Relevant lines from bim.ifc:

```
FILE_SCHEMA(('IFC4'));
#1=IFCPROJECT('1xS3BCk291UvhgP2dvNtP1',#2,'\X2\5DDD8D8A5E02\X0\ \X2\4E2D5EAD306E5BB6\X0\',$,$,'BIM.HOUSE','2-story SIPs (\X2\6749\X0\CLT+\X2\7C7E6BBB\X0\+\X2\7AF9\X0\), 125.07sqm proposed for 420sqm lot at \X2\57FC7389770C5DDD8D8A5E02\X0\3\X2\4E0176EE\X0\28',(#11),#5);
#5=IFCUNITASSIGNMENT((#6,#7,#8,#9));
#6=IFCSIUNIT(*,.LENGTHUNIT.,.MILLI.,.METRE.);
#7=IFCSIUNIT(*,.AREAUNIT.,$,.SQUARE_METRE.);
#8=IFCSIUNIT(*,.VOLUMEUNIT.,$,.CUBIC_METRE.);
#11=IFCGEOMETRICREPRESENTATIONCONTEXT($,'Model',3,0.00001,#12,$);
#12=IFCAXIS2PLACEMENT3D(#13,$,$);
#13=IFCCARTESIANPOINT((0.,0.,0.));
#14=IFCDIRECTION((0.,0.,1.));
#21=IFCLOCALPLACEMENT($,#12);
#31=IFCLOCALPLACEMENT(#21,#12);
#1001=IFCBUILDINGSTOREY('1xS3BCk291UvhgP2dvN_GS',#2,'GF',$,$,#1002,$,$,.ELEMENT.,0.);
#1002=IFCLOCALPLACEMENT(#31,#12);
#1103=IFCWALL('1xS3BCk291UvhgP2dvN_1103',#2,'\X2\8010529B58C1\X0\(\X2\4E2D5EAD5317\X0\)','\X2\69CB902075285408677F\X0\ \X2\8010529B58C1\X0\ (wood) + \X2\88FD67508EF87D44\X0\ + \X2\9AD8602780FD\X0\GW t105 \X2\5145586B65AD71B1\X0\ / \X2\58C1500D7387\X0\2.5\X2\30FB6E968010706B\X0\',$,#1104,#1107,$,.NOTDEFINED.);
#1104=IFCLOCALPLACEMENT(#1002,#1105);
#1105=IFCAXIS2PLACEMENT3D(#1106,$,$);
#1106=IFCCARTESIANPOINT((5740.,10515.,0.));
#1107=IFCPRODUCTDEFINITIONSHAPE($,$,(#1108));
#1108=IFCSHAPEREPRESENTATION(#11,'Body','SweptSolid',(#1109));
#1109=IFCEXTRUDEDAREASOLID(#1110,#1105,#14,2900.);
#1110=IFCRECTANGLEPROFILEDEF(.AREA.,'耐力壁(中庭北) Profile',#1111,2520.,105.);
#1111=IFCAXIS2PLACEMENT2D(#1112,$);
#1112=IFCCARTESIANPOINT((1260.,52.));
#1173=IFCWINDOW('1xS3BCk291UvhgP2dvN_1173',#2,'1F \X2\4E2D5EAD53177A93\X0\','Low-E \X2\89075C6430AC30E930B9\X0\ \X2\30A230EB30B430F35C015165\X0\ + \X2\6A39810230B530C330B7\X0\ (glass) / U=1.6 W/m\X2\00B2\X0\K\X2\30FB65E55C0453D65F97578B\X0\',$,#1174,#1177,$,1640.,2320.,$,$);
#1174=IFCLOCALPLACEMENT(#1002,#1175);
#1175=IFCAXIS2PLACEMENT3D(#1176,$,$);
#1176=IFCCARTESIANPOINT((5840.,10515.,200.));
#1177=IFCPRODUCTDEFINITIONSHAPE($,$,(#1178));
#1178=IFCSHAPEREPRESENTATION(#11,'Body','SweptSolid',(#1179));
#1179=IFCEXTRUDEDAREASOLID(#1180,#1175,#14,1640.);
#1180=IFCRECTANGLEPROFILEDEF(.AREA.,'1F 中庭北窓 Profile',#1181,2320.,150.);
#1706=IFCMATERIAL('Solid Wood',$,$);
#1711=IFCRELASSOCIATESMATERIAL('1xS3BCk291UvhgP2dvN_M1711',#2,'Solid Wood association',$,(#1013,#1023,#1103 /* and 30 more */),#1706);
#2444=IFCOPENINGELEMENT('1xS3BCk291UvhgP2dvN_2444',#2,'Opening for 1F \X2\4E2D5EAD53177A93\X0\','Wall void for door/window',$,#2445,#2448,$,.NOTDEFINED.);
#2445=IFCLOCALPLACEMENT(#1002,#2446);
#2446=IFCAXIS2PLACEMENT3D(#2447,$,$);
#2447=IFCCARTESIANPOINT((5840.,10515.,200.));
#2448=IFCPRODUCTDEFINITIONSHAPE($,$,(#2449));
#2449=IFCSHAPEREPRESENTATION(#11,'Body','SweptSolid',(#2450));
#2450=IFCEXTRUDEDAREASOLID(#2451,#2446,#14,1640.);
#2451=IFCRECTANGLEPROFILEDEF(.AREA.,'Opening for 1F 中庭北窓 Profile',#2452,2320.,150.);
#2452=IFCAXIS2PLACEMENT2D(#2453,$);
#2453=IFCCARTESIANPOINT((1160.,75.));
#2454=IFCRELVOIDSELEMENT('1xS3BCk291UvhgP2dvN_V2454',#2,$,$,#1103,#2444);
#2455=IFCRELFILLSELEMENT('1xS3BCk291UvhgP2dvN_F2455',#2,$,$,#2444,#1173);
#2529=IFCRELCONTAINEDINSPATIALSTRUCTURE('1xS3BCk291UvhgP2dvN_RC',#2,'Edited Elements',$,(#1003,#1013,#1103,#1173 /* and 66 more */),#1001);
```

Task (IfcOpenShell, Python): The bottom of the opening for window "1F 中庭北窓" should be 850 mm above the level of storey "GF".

```python
import numpy as np
import ifcopenshell
import ifcopenshell.api.geometry
import ifcopenshell.geom
import ifcopenshell.util.element
import ifcopenshell.util.placement
import ifcopenshell.util.shape
import ifcopenshell.util.unit

model = ifcopenshell.open("bim.ifc")
unit_scale = ifcopenshell.util.unit.calculate_unit_scale(model)

window = model.by_id(1173)
opening = window.FillsVoids[0].RelatingOpeningElement
storey = ifcopenshell.util.element.get_container(window, ifc_class="IfcBuildingStorey")
level = ifcopenshell.util.placement.get_local_placement(storey.ObjectPlacement)[2, 3]

# The opening's origin need not be at the sill, so measure its lowest point.
shape = ifcopenshell.geom.create_shape(ifcopenshell.geom.settings(), opening)
bottom = ifcopenshell.util.shape.get_shape_bottom_elevation(shape, shape.geometry) / unit_scale
dz = level + 850.0 - bottom

shift = np.array([0.0, 0.0, dz])
# The window is not placed relative to its opening, so move both.
for product in (opening, window):
    matrix = ifcopenshell.util.placement.get_local_placement(product.ObjectPlacement)
    matrix[:3, 3] += shift
    ifcopenshell.api.geometry.edit_object_placement(model, product=product, matrix=matrix, is_si=False)

print(f"moved by {dz * unit_scale:+.3f} m")

model.write("bim_v2.ifc")
```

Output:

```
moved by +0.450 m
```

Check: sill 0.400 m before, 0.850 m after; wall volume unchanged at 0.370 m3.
